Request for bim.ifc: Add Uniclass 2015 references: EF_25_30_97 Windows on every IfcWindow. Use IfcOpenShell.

First a look at what the model holds.

```python
import ifcopenshell

model = ifcopenshell.open("bim.ifc")
print(model.schema)
print("classifications:", [c.Name for c in model.by_type("IfcClassification")])
for ifc_class in ("IfcDoor", "IfcRoof", "IfcStair", "IfcWall", "IfcWindow"):
    print(ifc_class, len(model.by_type(ifc_class)))
```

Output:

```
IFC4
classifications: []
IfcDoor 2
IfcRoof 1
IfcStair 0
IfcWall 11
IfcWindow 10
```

```python
import ifcopenshell
import ifcopenshell.api.classification

model = ifcopenshell.open("bim.ifc")

system = ifcopenshell.api.classification.add_classification(model, classification="Uniclass 2015")

codes = {
    "IfcWindow": ("EF_25_30_97", "Windows"),
}
for ifc_class, (code, name) in codes.items():
    products = model.by_type(ifc_class)
    ifcopenshell.api.classification.add_reference(
        model, products=products, classification=system, identification=code, name=name
    )
    print(code, len(products))

model.write("bim_rev.ifc")
```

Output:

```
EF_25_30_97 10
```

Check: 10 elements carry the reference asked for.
